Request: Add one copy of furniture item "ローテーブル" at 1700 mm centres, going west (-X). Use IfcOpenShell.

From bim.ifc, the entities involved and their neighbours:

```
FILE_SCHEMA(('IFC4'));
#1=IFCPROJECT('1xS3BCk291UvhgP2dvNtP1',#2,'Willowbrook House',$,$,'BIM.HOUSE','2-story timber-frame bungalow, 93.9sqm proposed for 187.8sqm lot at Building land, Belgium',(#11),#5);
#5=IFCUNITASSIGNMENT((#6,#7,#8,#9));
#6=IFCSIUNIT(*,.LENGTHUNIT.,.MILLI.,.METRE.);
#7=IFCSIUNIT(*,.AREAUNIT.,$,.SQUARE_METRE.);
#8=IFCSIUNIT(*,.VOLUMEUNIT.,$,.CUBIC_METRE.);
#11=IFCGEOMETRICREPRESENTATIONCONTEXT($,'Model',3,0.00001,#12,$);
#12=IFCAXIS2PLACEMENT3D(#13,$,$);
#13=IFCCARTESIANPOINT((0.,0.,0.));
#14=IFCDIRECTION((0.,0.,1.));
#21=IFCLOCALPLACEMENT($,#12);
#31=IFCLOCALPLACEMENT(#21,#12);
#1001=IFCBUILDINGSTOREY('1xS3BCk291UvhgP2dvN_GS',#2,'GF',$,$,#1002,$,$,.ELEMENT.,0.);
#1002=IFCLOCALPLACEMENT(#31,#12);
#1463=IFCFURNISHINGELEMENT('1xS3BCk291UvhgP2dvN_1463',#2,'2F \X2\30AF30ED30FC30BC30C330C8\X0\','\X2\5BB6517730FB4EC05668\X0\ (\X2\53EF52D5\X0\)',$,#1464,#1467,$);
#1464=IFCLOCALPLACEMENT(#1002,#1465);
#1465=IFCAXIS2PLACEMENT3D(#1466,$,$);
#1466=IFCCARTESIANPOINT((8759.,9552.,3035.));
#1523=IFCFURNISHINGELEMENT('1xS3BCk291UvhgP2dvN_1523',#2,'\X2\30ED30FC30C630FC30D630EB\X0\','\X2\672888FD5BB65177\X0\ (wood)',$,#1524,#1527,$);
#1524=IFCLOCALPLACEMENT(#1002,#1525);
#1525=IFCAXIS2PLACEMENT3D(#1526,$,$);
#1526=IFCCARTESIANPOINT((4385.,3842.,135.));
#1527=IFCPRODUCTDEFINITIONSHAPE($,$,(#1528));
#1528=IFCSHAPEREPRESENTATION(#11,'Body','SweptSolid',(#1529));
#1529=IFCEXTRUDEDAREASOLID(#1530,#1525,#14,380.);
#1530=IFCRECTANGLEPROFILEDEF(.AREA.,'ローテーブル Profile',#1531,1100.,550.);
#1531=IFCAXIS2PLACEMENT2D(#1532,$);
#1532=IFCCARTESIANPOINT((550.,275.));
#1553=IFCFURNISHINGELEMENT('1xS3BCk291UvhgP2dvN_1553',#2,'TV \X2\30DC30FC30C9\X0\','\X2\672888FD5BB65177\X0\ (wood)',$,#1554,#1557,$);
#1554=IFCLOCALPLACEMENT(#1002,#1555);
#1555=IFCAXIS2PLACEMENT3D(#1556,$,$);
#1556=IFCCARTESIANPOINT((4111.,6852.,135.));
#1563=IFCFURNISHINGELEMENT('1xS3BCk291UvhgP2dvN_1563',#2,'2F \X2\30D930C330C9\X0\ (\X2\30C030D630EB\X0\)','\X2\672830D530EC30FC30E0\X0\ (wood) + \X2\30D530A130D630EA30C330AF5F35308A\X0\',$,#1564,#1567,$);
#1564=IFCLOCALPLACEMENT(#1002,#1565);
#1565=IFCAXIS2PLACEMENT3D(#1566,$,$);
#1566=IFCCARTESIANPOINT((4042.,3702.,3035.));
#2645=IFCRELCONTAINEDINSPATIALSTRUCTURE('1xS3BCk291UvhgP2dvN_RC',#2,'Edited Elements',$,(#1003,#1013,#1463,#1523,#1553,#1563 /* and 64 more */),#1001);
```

```python
import numpy as np
import ifcopenshell
import ifcopenshell.api.geometry
import ifcopenshell.api.root
import ifcopenshell.util.element
import ifcopenshell.util.placement

model = ifcopenshell.open("bim.ifc")


def reuse_history(source, copy):
    """copy_class also copies each property set's owner history, people and application; keep the originals."""
    for rel in copy.IsDefinedBy:
        if rel.is_a("IfcRelDefinesByProperties") and (history := rel.RelatingPropertyDefinition.OwnerHistory):
            rel.RelatingPropertyDefinition.OwnerHistory = source.OwnerHistory
            ifcopenshell.util.element.remove_deep2(model, history)


source = model.by_guid("1xS3BCk291UvhgP2dvN_1523")
base = ifcopenshell.util.placement.get_local_placement(source.ObjectPlacement)
step = np.array([-1.0, 0.0, 0.0]) * 1700.0

for i in range(1, 2):
    copy = ifcopenshell.api.root.copy_class(model, product=source)
    copy.Representation = ifcopenshell.util.element.copy_deep(
        model, source.Representation, exclude=["IfcGeometricRepresentationContext", "IfcRepresentationMap"]
    )
    reuse_history(source, copy)
    matrix = base.copy()
    matrix[:3, 3] += i * step
    print("added at", matrix[:3, 3].round(3) + 0.0)
    ifcopenshell.api.geometry.edit_object_placement(model, product=copy, matrix=matrix, is_si=False)

model.write("bim_edited.ifc")
```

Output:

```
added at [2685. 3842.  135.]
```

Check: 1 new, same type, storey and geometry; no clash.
